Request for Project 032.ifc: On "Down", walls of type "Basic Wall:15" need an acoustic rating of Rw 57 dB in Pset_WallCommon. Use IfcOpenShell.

First a look at what the model holds.

```python
import ifcopenshell
import ifcopenshell.util.element

model = ifcopenshell.open("Project 032.ifc")
print(model.schema)
storey = next(s for s in model.by_type("IfcBuildingStorey") if s.Name == "Down")
walls = [e for e in ifcopenshell.util.element.get_decomposition(storey) if e.is_a("IfcWall")]
seen = {}
for e in walls:
    element_type = ifcopenshell.util.element.get_type(e)
    key = (element_type.Name if element_type != e and element_type else None, ifcopenshell.util.element.get_pset(e, "Pset_WallCommon", "AcousticRating"))
    seen[key] = seen.get(key, 0) + 1
for (name, value), count in sorted(seen.items(), key=str):
    print(count, "x", name, "|", value)
```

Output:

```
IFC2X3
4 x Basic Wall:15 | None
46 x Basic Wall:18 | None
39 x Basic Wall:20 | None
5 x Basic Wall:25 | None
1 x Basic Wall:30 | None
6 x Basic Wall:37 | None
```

```python
import ifcopenshell
import ifcopenshell.api.pset
import ifcopenshell.util.element

model = ifcopenshell.open("Project 032.ifc")

storey = next(s for s in model.by_type("IfcBuildingStorey") if s.Name == "Down")
walls = [e for e in ifcopenshell.util.element.get_decomposition(storey) if e.is_a("IfcWall")]

count = 0
for e in walls:
    element_type = ifcopenshell.util.element.get_type(e)
    if element_type in (None, e) or element_type.Name != "Basic Wall:15":
        continue
    # add_pset returns the element's existing set when there is one.
    pset = ifcopenshell.api.pset.add_pset(model, product=e, name="Pset_WallCommon")
    ifcopenshell.api.pset.edit_pset(model, pset=pset, properties={"AcousticRating": "Rw 57 dB"})
    count += 1

print(count, "walls updated")

model.write("Project 032_rev.ifc")
```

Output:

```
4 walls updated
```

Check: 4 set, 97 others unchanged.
